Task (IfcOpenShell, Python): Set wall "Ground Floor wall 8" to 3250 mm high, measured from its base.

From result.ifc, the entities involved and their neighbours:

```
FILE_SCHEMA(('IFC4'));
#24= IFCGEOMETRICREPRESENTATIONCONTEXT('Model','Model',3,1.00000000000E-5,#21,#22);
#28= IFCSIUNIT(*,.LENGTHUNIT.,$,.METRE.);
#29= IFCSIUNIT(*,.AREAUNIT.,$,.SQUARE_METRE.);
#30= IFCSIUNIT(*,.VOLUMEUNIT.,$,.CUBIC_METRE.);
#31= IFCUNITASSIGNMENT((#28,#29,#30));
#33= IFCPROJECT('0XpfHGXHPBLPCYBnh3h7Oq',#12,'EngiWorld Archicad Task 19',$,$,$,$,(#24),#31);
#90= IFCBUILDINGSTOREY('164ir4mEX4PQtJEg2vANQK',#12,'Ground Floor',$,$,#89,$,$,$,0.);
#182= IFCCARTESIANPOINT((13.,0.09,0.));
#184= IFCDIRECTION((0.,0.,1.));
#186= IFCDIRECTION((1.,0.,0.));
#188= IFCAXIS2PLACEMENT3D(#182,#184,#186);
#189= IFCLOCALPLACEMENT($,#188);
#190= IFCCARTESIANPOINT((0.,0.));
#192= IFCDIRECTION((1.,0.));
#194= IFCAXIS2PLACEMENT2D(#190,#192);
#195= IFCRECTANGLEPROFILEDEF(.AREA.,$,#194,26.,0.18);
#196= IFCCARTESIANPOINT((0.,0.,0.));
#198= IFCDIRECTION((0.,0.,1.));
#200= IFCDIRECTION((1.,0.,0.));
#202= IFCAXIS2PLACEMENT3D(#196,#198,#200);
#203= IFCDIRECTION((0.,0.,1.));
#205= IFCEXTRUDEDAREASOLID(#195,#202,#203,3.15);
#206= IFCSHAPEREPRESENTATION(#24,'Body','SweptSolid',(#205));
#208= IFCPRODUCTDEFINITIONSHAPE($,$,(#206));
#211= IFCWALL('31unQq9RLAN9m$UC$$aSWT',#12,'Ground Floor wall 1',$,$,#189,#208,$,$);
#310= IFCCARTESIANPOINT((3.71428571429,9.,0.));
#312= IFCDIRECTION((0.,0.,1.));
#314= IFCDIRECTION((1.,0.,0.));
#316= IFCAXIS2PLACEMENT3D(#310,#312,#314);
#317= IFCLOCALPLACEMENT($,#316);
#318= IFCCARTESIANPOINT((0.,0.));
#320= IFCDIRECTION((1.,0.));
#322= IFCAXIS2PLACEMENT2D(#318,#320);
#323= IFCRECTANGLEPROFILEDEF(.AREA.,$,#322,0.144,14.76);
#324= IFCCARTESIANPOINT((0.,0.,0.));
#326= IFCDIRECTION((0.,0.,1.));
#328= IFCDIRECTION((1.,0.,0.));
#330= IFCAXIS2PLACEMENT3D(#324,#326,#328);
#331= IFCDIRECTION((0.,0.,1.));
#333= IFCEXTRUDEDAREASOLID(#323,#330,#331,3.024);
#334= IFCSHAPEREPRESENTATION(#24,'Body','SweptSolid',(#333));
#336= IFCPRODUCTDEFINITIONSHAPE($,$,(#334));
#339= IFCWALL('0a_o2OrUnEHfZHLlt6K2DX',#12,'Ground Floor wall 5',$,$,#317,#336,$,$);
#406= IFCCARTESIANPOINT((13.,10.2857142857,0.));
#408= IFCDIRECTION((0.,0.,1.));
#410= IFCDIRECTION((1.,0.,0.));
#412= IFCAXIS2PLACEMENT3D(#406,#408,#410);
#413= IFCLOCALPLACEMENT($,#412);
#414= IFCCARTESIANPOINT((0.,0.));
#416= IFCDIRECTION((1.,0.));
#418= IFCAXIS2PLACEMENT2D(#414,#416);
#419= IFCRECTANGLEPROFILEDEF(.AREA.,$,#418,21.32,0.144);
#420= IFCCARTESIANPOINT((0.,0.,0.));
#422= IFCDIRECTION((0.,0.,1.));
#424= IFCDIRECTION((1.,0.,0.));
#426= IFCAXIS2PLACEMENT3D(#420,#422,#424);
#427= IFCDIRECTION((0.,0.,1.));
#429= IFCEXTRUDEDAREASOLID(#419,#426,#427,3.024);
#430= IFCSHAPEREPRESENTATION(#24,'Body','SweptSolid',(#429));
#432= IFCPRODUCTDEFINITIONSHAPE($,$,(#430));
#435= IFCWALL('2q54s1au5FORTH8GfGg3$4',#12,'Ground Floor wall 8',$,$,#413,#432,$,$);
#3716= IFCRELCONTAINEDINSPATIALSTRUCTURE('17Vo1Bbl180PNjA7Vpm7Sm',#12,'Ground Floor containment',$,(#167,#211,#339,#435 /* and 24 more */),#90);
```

```python
import ifcopenshell
import ifcopenshell.geom
import ifcopenshell.util.shape
import ifcopenshell.util.unit

model = ifcopenshell.open("result.ifc")
unit_scale = ifcopenshell.util.unit.calculate_unit_scale(model)
settings = ifcopenshell.geom.settings()


def volume(element):
    """Net volume in cubic metres, openings subtracted."""
    shape = ifcopenshell.geom.create_shape(settings, element)
    return ifcopenshell.util.shape.get_volume(shape.geometry)


wall = model.by_guid("2q54s1au5FORTH8GfGg3$4")
before = volume(wall)

body = next(r for r in wall.Representation.Representations if r.RepresentationIdentifier == "Body")
solid = body.Items[0]
old_height = solid.Depth
solid.Depth = 3.25 / unit_scale
after = volume(wall)

print(f"height {old_height:g} -> {solid.Depth:g}, volume {before:.3f} -> {after:.3f} m3")

model.write("result_v2.ifc")
```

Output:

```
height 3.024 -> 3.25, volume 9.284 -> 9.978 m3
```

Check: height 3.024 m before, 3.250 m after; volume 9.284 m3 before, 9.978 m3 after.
